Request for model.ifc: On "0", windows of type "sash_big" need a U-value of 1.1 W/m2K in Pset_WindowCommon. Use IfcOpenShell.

First a look at what the model holds.

```python
import ifcopenshell
import ifcopenshell.util.element

model = ifcopenshell.open("model.ifc")
print(model.schema)
storey = next(s for s in model.by_type("IfcBuildingStorey") if s.Name == "0")
windows = [e for e in ifcopenshell.util.element.get_decomposition(storey) if e.is_a("IfcWindow")]
seen = {}
for e in windows:
    element_type = ifcopenshell.util.element.get_type(e)
    key = (element_type.Name if element_type != e and element_type else None, ifcopenshell.util.element.get_pset(e, "Pset_WindowCommon", "ThermalTransmittance"))
    seen[key] = seen.get(key, 0) + 1
for (name, value), count in sorted(seen.items(), key=str):
    print(count, "x", name, "|", value)
```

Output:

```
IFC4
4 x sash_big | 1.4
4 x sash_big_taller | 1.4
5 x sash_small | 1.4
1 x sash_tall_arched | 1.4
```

```python
import ifcopenshell
import ifcopenshell.api.pset
import ifcopenshell.util.element

model = ifcopenshell.open("model.ifc")

storey = next(s for s in model.by_type("IfcBuildingStorey") if s.Name == "0")
windows = [e for e in ifcopenshell.util.element.get_decomposition(storey) if e.is_a("IfcWindow")]

count = 0
for e in windows:
    element_type = ifcopenshell.util.element.get_type(e)
    if element_type in (None, e) or element_type.Name != "sash_big":
        continue
    # add_pset returns the element's existing set when there is one.
    pset = ifcopenshell.api.pset.add_pset(model, product=e, name="Pset_WindowCommon")
    ifcopenshell.api.pset.edit_pset(model, pset=pset, properties={"ThermalTransmittance": 1.1})
    count += 1

print(count, "windows updated")

model.write("model_edited.ifc")
```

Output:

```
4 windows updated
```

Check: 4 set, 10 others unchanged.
